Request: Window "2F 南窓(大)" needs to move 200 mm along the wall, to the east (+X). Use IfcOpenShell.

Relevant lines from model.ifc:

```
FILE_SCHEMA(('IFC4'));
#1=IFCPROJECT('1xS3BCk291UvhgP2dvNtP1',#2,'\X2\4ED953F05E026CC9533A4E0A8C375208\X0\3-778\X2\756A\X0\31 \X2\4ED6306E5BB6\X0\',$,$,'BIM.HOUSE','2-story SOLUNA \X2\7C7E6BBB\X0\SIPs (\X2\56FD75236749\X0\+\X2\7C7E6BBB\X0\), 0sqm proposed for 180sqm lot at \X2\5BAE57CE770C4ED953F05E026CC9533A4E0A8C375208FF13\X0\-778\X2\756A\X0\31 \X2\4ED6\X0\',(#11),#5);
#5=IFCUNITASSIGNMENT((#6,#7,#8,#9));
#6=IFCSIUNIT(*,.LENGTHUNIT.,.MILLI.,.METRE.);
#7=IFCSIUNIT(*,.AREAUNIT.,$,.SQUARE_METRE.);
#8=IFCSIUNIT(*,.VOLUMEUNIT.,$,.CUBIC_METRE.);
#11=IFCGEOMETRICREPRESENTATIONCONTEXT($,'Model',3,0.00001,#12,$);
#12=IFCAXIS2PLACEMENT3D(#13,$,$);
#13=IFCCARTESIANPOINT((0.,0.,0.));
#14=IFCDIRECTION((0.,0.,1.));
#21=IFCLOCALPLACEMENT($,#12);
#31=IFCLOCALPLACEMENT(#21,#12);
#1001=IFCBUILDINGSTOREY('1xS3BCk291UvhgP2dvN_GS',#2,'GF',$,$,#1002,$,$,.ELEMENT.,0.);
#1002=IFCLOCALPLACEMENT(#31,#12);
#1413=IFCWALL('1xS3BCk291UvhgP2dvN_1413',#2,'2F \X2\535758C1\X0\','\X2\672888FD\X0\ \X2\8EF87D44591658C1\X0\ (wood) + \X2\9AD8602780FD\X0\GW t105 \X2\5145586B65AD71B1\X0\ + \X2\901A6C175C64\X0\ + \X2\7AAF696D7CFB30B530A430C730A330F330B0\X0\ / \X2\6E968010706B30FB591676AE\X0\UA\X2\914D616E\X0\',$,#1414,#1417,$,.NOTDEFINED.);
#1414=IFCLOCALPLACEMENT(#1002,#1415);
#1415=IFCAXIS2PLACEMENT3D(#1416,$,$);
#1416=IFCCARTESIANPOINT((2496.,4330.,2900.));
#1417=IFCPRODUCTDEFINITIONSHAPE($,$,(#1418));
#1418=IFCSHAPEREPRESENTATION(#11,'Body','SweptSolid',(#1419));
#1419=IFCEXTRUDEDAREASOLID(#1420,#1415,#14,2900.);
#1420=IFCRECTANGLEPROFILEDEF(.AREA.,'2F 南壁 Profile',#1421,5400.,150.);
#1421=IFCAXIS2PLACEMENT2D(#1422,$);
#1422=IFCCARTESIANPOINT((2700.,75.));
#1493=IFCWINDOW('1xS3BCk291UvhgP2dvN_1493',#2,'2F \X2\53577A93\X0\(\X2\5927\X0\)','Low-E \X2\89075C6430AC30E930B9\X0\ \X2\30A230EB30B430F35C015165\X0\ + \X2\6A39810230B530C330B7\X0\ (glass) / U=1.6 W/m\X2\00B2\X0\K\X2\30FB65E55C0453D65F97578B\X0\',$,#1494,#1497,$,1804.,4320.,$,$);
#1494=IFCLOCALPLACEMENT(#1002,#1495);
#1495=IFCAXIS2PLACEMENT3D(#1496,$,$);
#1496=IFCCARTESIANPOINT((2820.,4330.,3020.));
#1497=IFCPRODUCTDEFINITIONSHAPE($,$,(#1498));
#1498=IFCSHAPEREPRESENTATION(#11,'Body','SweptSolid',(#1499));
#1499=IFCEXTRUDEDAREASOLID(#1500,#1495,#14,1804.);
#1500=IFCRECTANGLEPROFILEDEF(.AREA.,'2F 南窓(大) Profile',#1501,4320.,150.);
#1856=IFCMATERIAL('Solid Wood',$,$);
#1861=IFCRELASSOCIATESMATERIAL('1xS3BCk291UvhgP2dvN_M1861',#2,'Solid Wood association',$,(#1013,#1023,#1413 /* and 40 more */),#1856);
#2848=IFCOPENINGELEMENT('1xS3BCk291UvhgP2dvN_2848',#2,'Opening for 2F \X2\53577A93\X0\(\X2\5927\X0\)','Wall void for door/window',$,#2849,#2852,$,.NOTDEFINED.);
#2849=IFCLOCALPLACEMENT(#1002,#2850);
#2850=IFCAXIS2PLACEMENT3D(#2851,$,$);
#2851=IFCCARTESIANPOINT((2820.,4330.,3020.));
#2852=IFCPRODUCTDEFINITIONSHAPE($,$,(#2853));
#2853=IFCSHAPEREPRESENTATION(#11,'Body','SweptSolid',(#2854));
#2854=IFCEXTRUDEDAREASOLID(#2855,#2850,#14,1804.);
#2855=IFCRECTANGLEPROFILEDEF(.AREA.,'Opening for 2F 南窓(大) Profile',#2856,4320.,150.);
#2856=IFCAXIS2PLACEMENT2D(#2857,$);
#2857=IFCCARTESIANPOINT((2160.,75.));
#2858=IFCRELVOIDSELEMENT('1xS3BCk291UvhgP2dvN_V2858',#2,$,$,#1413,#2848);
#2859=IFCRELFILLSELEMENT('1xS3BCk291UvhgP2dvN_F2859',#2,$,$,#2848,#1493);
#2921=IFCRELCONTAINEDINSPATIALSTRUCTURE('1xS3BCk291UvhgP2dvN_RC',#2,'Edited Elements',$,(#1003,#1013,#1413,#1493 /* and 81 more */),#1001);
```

```python
import ifcopenshell
import ifcopenshell.api.geometry
import ifcopenshell.util.placement
import ifcopenshell.util.unit

model = ifcopenshell.open("model.ifc")
unit_scale = ifcopenshell.util.unit.calculate_unit_scale(model)

window = model.by_guid("1xS3BCk291UvhgP2dvN_1493")
opening = window.FillsVoids[0].RelatingOpeningElement
wall = opening.VoidsElements[0].RelatingBuildingElement

wall_matrix = ifcopenshell.util.placement.get_local_placement(wall.ObjectPlacement)
shift = wall_matrix[:3, 0] * 0.2 / unit_scale
before = ifcopenshell.util.placement.get_local_placement(window.ObjectPlacement)[:3, 3].copy()

# The window is not placed relative to its opening, so move both.
for product in (opening, window):
    matrix = ifcopenshell.util.placement.get_local_placement(product.ObjectPlacement)
    matrix[:3, 3] += shift
    ifcopenshell.api.geometry.edit_object_placement(model, product=product, matrix=matrix, is_si=False)

after = ifcopenshell.util.placement.get_local_placement(window.ObjectPlacement)[:3, 3]
print("window moved by", (after - before).round(3) + 0.0)

model.write("model_edited.ifc")
```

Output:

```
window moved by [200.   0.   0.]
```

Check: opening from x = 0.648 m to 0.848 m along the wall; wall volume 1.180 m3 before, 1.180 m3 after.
